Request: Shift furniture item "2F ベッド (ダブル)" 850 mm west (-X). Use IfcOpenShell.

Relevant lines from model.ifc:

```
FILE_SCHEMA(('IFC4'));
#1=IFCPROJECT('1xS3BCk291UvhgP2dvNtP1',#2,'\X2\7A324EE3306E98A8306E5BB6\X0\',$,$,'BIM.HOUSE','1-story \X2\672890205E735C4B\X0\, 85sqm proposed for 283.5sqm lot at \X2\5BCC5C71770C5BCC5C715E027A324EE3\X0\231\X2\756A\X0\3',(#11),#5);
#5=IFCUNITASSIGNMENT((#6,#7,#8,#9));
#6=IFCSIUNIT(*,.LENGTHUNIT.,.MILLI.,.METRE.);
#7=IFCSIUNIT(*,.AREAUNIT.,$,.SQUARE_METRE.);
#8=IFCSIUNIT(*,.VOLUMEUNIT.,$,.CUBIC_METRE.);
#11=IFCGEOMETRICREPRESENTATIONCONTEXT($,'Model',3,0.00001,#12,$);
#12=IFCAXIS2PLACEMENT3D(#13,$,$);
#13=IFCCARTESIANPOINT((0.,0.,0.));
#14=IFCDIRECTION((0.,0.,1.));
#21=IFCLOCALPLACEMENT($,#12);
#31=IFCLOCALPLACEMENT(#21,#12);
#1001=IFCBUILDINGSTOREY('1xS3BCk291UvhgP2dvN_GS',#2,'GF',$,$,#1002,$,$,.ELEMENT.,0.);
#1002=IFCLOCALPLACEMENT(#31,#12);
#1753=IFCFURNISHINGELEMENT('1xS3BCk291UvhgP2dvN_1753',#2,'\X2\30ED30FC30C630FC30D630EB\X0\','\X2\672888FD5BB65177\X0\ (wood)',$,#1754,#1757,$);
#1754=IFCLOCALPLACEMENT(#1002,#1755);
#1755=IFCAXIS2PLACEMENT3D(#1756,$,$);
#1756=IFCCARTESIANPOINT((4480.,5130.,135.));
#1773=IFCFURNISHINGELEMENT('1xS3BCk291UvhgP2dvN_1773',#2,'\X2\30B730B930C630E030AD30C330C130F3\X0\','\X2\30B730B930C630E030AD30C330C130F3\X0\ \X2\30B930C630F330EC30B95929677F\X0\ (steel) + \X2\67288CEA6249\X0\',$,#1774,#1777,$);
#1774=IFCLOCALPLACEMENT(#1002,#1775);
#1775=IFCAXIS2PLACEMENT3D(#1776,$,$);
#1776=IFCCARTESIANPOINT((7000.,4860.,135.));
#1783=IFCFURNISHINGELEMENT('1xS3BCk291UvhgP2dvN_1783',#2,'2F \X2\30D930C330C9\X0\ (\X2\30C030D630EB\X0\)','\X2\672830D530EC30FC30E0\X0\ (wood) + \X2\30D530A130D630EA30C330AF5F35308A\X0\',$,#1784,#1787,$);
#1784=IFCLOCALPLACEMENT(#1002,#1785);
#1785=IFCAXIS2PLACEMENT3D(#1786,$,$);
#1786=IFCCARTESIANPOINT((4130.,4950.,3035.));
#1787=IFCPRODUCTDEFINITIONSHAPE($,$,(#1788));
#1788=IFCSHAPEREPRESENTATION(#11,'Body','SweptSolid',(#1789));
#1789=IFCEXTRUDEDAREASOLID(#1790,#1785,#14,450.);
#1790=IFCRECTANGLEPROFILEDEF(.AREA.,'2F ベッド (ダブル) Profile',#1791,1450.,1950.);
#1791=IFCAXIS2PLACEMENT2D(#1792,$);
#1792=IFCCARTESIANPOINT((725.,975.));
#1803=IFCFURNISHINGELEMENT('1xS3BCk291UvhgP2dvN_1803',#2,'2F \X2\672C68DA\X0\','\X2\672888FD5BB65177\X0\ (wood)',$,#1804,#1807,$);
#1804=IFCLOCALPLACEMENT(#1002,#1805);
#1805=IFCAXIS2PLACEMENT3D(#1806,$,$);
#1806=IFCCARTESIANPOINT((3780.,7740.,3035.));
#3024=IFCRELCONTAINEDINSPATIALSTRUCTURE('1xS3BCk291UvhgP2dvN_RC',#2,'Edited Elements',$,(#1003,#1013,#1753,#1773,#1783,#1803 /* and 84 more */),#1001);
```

```python
import ifcopenshell
import ifcopenshell.api.geometry
import ifcopenshell.util.placement
import ifcopenshell.util.unit

model = ifcopenshell.open("model.ifc")
unit_scale = ifcopenshell.util.unit.calculate_unit_scale(model)

item = model.by_guid("1xS3BCk291UvhgP2dvN_1783")
matrix = ifcopenshell.util.placement.get_local_placement(item.ObjectPlacement)
matrix[0, 3] -= 0.85 / unit_scale
ifcopenshell.api.geometry.edit_object_placement(model, product=item, matrix=matrix, is_si=False)

print(ifcopenshell.util.placement.get_local_placement(item.ObjectPlacement).round(3) + 0.0)

model.write("model-out.ifc")
```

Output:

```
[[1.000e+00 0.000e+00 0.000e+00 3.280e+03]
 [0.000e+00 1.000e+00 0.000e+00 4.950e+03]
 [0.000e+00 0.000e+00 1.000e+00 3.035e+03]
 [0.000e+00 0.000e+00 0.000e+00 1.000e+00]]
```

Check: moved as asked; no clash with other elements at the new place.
